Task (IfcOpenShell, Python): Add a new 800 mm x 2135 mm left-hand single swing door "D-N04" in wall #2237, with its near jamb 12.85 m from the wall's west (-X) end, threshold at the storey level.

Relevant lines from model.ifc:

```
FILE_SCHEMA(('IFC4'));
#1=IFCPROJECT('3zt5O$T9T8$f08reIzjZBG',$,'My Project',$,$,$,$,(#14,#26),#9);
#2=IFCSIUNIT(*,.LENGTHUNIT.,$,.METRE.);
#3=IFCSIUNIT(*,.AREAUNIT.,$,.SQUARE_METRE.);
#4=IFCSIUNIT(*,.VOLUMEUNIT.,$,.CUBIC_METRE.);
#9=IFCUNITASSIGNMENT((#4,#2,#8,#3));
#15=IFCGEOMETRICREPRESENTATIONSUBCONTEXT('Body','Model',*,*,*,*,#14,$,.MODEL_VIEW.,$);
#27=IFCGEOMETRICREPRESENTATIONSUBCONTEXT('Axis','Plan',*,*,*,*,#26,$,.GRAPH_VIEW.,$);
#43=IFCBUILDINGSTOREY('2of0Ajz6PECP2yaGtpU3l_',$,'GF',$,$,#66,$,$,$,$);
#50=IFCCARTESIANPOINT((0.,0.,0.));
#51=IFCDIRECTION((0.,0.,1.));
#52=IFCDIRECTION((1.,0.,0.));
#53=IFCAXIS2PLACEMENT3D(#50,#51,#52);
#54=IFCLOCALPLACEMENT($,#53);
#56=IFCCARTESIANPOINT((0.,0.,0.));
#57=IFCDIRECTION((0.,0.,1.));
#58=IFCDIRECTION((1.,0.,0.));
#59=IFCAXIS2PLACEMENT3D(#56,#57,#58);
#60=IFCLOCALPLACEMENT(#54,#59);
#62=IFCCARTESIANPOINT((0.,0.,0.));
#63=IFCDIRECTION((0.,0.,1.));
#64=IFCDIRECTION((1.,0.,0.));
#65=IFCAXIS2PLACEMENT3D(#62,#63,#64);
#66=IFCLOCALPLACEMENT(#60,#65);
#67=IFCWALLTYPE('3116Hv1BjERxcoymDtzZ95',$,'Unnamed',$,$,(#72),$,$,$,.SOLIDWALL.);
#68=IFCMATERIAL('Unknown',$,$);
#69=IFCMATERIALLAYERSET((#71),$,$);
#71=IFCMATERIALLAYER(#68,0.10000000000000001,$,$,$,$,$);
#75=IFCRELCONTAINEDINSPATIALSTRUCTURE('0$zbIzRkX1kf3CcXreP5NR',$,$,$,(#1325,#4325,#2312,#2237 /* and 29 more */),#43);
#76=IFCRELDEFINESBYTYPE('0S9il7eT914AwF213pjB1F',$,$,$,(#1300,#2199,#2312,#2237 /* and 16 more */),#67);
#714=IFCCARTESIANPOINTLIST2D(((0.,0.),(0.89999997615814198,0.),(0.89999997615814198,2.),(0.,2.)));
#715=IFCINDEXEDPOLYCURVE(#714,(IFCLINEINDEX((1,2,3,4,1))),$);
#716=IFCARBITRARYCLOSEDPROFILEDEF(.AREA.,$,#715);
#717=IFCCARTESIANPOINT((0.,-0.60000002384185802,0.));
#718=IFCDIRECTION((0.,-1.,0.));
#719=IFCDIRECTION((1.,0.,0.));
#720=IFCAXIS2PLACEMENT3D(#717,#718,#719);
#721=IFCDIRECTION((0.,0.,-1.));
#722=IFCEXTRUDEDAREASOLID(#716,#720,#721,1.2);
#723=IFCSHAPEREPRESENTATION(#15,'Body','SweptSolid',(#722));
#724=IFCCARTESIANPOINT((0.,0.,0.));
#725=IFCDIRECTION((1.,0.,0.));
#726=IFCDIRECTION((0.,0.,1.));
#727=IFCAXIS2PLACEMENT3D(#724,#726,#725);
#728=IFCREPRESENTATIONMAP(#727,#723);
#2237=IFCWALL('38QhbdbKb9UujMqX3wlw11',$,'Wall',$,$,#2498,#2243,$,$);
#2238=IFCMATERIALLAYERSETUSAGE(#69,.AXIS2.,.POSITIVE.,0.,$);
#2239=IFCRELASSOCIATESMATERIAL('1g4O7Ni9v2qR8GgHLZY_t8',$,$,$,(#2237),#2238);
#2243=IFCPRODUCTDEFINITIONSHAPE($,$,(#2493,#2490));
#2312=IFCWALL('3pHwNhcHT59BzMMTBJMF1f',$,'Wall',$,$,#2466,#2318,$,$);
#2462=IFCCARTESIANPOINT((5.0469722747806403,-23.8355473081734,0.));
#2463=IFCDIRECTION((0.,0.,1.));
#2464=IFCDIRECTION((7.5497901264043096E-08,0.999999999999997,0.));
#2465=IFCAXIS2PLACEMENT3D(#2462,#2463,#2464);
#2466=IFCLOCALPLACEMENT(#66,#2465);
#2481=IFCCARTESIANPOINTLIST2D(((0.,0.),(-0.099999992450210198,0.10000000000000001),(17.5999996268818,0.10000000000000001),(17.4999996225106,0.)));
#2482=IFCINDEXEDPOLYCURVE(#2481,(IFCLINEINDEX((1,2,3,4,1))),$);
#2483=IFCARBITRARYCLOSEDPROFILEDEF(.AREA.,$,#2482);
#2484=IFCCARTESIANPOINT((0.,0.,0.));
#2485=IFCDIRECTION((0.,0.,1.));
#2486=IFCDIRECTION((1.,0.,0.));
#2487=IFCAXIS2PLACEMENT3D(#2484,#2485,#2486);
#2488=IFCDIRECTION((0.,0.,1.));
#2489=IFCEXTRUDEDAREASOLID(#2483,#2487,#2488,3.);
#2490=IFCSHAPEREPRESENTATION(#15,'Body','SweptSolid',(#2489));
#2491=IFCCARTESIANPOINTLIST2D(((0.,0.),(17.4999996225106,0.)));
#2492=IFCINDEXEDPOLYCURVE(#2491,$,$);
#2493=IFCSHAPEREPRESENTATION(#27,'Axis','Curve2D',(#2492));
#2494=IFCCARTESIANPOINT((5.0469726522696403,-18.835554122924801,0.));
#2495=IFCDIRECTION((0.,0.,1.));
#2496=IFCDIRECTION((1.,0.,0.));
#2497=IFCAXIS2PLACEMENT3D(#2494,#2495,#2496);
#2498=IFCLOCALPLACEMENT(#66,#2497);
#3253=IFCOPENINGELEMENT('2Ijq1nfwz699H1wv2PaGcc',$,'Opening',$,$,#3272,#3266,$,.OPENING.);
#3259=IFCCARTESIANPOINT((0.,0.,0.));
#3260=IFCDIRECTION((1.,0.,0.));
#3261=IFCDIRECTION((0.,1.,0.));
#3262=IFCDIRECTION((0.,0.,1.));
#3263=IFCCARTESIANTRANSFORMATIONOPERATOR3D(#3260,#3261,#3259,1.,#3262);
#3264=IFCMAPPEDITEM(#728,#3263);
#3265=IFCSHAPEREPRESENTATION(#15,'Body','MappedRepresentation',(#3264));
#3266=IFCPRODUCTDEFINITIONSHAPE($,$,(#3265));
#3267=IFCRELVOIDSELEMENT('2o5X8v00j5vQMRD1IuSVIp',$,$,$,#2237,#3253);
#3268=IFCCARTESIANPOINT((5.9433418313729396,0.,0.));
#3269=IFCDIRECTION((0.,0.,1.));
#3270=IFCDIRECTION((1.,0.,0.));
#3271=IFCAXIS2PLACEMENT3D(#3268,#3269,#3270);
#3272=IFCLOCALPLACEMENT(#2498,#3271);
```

```python
import numpy as np
import ifcopenshell
import ifcopenshell.api.feature
import ifcopenshell.api.geometry
import ifcopenshell.api.root
import ifcopenshell.api.spatial
import ifcopenshell.geom
import ifcopenshell.util.element
import ifcopenshell.util.placement
import ifcopenshell.util.representation
import ifcopenshell.util.shape
import ifcopenshell.util.unit

model = ifcopenshell.open("model.ifc")
unit_scale = ifcopenshell.util.unit.calculate_unit_scale(model)
settings = ifcopenshell.geom.settings()


def volume(element):
    """Net volume in cubic metres, openings subtracted."""
    shape = ifcopenshell.geom.create_shape(settings, element)
    return ifcopenshell.util.shape.get_volume(shape.geometry)


wall = model.by_guid("38QhbdbKb9UujMqX3wlw11")
storey = ifcopenshell.util.element.get_container(wall, ifc_class="IfcBuildingStorey")
context = ifcopenshell.util.representation.get_context(model, "Model", "Body", "MODEL_VIEW")
before = volume(wall)

width, height, from_end, sill = 0.8, 2.135, 12.85, 0.0  # metres

# The wall runs along its own X axis, and the end named is its -X end.
wall_shape = ifcopenshell.geom.create_shape(settings, wall)
x, y, z = ifcopenshell.util.shape.get_vertices(wall_shape.geometry).T
start = x.min() + from_end
face, thickness = float(y.min()), float(y.max() - y.min())
wall_matrix = ifcopenshell.util.placement.get_local_placement(wall.ObjectPlacement)
level = ifcopenshell.util.placement.get_local_placement(storey.ObjectPlacement)[2, 3]


def in_wall(x, y):
    """Placement at x, y metres in the wall's axes, at sill height."""
    matrix = wall_matrix.copy()
    matrix[:, 3] = wall_matrix @ np.array([x / unit_scale, y / unit_scale, 0.0, 1.0])
    matrix[2, 3] = level + sill / unit_scale
    return matrix


# Opening: a box that overshoots both wall faces by 50 mm.
opening = ifcopenshell.api.root.create_entity(model, ifc_class="IfcOpeningElement", predefined_type="OPENING")
box = ifcopenshell.api.geometry.add_wall_representation(
    model, context=context, length=width, height=height, thickness=thickness + 0.1
)
ifcopenshell.api.geometry.assign_representation(model, product=opening, representation=box)
ifcopenshell.api.geometry.edit_object_placement(model, product=opening, matrix=in_wall(start, face - 0.05), is_si=False)
ifcopenshell.api.feature.add_feature(model, feature=opening, element=wall)

door = ifcopenshell.api.root.create_entity(model, ifc_class="IfcDoor", name="D-N04", predefined_type="DOOR")
door.OverallWidth, door.OverallHeight = width / unit_scale, height / unit_scale
door.OperationType = "SINGLE_SWING_LEFT"
body = ifcopenshell.api.geometry.add_door_representation(
    model,
    context=context,
    overall_width=door.OverallWidth,
    overall_height=door.OverallHeight,
    operation_type="SINGLE_SWING_LEFT",
    lining_properties={"LiningDepth": thickness / unit_scale, "ThresholdDepth": thickness / unit_scale},
)
ifcopenshell.api.geometry.assign_representation(model, product=door, representation=body)
ifcopenshell.api.spatial.assign_container(model, products=[door], relating_structure=storey)
ifcopenshell.api.feature.add_filling(model, opening=opening, element=door)

# The lining spans the wall, so the door starts at the wall face.
ifcopenshell.api.geometry.edit_object_placement(model, product=door, matrix=in_wall(start, face), is_si=False)

after = volume(wall)

print(f"wall volume {before:.3f} -> {after:.3f} m3")

model.write("model_v2.ifc")
```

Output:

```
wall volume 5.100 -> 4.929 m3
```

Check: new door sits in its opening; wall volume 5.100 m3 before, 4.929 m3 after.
